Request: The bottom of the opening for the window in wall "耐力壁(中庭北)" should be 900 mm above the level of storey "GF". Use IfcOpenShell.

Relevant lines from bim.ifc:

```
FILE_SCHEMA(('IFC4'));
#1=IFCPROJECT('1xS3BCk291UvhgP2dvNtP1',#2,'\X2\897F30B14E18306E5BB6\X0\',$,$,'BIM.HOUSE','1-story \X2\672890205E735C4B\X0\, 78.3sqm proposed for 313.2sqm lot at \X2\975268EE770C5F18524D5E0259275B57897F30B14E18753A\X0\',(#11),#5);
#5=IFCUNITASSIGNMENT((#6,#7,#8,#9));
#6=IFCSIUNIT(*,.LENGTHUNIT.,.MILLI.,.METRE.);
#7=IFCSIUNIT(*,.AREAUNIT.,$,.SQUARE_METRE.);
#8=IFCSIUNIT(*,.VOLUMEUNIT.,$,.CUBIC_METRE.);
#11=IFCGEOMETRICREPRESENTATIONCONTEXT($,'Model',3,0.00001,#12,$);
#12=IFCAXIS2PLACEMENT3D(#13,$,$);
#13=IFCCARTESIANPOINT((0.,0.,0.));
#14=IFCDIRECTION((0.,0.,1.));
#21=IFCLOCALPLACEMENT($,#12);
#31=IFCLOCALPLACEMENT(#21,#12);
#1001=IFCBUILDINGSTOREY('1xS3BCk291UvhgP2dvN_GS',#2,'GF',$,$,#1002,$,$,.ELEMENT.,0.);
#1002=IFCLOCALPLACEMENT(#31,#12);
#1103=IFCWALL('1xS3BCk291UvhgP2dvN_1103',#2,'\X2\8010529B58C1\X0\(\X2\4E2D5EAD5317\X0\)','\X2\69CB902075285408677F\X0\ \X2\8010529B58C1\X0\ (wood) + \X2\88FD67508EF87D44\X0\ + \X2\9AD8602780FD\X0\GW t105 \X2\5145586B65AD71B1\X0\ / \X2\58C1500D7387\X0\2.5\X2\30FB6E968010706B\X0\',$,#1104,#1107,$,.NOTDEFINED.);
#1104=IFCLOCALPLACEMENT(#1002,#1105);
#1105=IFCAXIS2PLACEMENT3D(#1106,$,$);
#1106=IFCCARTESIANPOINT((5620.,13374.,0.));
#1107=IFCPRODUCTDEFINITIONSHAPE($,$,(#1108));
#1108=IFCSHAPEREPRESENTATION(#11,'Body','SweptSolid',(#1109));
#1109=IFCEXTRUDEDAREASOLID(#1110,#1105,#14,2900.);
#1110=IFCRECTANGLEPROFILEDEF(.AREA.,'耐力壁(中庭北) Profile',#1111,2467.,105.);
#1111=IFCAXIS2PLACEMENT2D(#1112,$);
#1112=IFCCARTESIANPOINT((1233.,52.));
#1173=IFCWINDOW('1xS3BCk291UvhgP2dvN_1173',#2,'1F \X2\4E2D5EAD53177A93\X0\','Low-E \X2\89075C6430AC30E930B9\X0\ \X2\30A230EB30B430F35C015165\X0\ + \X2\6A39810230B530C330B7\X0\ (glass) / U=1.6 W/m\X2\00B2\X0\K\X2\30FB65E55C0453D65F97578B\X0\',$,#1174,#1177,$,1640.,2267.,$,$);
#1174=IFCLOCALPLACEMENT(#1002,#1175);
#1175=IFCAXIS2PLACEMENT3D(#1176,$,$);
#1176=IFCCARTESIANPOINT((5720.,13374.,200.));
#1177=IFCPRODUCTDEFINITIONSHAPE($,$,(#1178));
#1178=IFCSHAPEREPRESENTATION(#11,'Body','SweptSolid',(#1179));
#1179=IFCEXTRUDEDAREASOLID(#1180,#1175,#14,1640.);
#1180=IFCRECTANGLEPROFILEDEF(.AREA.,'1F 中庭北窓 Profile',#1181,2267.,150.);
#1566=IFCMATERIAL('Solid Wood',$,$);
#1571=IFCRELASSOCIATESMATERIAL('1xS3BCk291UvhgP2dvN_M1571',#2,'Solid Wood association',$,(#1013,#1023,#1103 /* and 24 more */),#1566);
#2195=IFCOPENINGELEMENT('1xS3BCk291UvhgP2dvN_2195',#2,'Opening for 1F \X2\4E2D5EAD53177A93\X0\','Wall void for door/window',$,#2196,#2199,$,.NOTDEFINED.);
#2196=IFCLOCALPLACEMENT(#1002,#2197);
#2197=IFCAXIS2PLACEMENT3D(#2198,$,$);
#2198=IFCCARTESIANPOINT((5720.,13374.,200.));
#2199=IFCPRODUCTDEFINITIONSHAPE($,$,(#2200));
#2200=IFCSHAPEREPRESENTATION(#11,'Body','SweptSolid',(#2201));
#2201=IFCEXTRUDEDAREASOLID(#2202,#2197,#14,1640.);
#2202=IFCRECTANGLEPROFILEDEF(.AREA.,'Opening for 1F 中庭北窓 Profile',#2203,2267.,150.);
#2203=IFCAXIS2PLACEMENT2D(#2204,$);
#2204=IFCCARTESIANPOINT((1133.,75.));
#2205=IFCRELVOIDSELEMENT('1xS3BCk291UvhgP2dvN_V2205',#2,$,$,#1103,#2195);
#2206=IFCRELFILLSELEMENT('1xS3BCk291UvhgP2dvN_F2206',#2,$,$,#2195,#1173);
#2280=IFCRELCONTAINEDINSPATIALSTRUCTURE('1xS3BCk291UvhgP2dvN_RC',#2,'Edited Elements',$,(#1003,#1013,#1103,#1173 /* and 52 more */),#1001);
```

```python
import numpy as np
import ifcopenshell
import ifcopenshell.api.geometry
import ifcopenshell.geom
import ifcopenshell.util.element
import ifcopenshell.util.placement
import ifcopenshell.util.shape
import ifcopenshell.util.unit

model = ifcopenshell.open("bim.ifc")
unit_scale = ifcopenshell.util.unit.calculate_unit_scale(model)

window = model.by_guid("1xS3BCk291UvhgP2dvN_1173")
opening = window.FillsVoids[0].RelatingOpeningElement
storey = ifcopenshell.util.element.get_container(window, ifc_class="IfcBuildingStorey")
level = ifcopenshell.util.placement.get_local_placement(storey.ObjectPlacement)[2, 3]

# The opening's origin need not be at the sill, so measure its lowest point.
shape = ifcopenshell.geom.create_shape(ifcopenshell.geom.settings(), opening)
bottom = ifcopenshell.util.shape.get_shape_bottom_elevation(shape, shape.geometry) / unit_scale
dz = level + 0.9 / unit_scale - bottom

shift = np.array([0.0, 0.0, dz])
# The window is not placed relative to its opening, so move both.
for product in (opening, window):
    matrix = ifcopenshell.util.placement.get_local_placement(product.ObjectPlacement)
    matrix[:3, 3] += shift
    ifcopenshell.api.geometry.edit_object_placement(model, product=product, matrix=matrix, is_si=False)

print(f"moved by {dz * unit_scale:+.3f} m")

model.write("bim-out.ifc")
```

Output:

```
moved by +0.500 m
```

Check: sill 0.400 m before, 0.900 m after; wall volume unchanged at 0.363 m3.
